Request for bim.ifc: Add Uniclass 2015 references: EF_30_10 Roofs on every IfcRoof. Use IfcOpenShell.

First a look at what the model holds.

```python
import ifcopenshell

model = ifcopenshell.open("bim.ifc")
print(model.schema)
print("classifications:", [c.Name for c in model.by_type("IfcClassification")])
for ifc_class in ("IfcDoor", "IfcRoof", "IfcStair", "IfcWall", "IfcWindow"):
    print(ifc_class, len(model.by_type(ifc_class)))
```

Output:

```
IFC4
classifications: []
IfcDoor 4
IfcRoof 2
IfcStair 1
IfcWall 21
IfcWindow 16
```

```python
import ifcopenshell
import ifcopenshell.api.classification

model = ifcopenshell.open("bim.ifc")

system = ifcopenshell.api.classification.add_classification(model, classification="Uniclass 2015")

codes = {
    "IfcRoof": ("EF_30_10", "Roofs"),
}
for ifc_class, (code, name) in codes.items():
    products = model.by_type(ifc_class)
    ifcopenshell.api.classification.add_reference(
        model, products=products, classification=system, identification=code, name=name
    )
    print(code, len(products))

model.write("bim_rev.ifc")
```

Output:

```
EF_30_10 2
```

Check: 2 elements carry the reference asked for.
